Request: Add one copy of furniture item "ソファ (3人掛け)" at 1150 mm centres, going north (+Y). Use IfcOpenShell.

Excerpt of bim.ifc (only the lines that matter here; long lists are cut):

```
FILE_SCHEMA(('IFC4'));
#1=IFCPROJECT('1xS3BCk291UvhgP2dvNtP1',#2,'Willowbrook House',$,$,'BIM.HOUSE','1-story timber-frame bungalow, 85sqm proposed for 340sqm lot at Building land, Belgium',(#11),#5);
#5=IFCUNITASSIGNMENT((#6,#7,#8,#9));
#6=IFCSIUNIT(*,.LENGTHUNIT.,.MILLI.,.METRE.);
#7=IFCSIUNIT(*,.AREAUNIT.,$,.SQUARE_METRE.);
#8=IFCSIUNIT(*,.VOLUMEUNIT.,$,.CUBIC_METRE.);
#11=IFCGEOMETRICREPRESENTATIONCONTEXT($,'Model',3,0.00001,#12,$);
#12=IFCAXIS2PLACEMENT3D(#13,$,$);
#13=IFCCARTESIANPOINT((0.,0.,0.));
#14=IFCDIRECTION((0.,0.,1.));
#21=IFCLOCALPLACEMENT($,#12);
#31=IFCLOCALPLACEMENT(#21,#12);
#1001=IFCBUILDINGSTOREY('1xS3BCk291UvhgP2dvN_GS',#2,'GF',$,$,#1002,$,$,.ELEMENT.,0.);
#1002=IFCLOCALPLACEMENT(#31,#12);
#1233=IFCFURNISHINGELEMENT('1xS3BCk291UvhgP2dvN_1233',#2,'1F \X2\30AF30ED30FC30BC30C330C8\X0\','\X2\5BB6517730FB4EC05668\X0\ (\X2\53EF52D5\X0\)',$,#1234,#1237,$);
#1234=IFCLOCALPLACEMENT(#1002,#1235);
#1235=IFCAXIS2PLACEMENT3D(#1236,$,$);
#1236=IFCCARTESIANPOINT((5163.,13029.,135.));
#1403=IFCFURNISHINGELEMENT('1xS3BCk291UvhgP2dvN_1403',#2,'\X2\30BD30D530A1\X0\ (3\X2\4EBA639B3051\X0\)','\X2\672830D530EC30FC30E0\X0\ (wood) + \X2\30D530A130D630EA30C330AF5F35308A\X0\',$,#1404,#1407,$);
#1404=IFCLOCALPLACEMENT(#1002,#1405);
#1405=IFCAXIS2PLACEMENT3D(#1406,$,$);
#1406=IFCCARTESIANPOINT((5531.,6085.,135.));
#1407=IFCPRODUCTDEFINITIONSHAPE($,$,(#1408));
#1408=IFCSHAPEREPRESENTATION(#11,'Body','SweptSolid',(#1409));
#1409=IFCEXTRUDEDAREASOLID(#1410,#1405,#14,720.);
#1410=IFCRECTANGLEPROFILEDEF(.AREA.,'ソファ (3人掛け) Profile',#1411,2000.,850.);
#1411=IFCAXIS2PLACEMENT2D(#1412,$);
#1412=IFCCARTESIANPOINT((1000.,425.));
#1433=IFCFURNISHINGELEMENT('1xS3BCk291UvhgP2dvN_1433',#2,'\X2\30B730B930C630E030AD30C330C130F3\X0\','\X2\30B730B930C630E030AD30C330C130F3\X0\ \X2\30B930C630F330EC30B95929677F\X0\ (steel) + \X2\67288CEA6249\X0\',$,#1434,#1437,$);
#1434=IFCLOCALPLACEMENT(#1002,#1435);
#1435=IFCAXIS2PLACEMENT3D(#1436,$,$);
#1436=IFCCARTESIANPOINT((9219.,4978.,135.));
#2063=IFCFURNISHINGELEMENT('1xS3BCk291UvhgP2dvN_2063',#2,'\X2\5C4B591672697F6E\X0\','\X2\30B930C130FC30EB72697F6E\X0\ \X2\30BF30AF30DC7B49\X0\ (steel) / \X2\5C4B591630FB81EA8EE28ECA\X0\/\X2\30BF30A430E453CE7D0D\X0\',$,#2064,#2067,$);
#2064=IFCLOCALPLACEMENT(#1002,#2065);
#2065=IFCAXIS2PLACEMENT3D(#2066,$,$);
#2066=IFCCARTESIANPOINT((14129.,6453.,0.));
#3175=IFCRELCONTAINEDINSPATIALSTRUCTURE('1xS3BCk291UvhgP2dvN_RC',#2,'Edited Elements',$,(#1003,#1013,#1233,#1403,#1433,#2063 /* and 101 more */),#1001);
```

```python
import numpy as np
import ifcopenshell
import ifcopenshell.api.geometry
import ifcopenshell.api.root
import ifcopenshell.util.element
import ifcopenshell.util.placement
import ifcopenshell.util.unit

model = ifcopenshell.open("bim.ifc")
unit_scale = ifcopenshell.util.unit.calculate_unit_scale(model)


def reuse_history(source, copy):
    """copy_class also copies each property set's owner history, people and application; keep the originals."""
    for rel in copy.IsDefinedBy:
        if rel.is_a("IfcRelDefinesByProperties") and (history := rel.RelatingPropertyDefinition.OwnerHistory):
            rel.RelatingPropertyDefinition.OwnerHistory = source.OwnerHistory
            ifcopenshell.util.element.remove_deep2(model, history)


source = model.by_guid("1xS3BCk291UvhgP2dvN_1403")
base = ifcopenshell.util.placement.get_local_placement(source.ObjectPlacement)
step = np.array([0.0, 1.0, 0.0]) * 1.15 / unit_scale

for i in range(1, 2):
    copy = ifcopenshell.api.root.copy_class(model, product=source)
    copy.Representation = ifcopenshell.util.element.copy_deep(
        model, source.Representation, exclude=["IfcGeometricRepresentationContext", "IfcRepresentationMap"]
    )
    reuse_history(source, copy)
    matrix = base.copy()
    matrix[:3, 3] += i * step
    print("added at", matrix[:3, 3].round(3) + 0.0)
    ifcopenshell.api.geometry.edit_object_placement(model, product=copy, matrix=matrix, is_si=False)

model.write("bim_rev.ifc")
```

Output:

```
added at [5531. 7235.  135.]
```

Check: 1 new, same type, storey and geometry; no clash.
